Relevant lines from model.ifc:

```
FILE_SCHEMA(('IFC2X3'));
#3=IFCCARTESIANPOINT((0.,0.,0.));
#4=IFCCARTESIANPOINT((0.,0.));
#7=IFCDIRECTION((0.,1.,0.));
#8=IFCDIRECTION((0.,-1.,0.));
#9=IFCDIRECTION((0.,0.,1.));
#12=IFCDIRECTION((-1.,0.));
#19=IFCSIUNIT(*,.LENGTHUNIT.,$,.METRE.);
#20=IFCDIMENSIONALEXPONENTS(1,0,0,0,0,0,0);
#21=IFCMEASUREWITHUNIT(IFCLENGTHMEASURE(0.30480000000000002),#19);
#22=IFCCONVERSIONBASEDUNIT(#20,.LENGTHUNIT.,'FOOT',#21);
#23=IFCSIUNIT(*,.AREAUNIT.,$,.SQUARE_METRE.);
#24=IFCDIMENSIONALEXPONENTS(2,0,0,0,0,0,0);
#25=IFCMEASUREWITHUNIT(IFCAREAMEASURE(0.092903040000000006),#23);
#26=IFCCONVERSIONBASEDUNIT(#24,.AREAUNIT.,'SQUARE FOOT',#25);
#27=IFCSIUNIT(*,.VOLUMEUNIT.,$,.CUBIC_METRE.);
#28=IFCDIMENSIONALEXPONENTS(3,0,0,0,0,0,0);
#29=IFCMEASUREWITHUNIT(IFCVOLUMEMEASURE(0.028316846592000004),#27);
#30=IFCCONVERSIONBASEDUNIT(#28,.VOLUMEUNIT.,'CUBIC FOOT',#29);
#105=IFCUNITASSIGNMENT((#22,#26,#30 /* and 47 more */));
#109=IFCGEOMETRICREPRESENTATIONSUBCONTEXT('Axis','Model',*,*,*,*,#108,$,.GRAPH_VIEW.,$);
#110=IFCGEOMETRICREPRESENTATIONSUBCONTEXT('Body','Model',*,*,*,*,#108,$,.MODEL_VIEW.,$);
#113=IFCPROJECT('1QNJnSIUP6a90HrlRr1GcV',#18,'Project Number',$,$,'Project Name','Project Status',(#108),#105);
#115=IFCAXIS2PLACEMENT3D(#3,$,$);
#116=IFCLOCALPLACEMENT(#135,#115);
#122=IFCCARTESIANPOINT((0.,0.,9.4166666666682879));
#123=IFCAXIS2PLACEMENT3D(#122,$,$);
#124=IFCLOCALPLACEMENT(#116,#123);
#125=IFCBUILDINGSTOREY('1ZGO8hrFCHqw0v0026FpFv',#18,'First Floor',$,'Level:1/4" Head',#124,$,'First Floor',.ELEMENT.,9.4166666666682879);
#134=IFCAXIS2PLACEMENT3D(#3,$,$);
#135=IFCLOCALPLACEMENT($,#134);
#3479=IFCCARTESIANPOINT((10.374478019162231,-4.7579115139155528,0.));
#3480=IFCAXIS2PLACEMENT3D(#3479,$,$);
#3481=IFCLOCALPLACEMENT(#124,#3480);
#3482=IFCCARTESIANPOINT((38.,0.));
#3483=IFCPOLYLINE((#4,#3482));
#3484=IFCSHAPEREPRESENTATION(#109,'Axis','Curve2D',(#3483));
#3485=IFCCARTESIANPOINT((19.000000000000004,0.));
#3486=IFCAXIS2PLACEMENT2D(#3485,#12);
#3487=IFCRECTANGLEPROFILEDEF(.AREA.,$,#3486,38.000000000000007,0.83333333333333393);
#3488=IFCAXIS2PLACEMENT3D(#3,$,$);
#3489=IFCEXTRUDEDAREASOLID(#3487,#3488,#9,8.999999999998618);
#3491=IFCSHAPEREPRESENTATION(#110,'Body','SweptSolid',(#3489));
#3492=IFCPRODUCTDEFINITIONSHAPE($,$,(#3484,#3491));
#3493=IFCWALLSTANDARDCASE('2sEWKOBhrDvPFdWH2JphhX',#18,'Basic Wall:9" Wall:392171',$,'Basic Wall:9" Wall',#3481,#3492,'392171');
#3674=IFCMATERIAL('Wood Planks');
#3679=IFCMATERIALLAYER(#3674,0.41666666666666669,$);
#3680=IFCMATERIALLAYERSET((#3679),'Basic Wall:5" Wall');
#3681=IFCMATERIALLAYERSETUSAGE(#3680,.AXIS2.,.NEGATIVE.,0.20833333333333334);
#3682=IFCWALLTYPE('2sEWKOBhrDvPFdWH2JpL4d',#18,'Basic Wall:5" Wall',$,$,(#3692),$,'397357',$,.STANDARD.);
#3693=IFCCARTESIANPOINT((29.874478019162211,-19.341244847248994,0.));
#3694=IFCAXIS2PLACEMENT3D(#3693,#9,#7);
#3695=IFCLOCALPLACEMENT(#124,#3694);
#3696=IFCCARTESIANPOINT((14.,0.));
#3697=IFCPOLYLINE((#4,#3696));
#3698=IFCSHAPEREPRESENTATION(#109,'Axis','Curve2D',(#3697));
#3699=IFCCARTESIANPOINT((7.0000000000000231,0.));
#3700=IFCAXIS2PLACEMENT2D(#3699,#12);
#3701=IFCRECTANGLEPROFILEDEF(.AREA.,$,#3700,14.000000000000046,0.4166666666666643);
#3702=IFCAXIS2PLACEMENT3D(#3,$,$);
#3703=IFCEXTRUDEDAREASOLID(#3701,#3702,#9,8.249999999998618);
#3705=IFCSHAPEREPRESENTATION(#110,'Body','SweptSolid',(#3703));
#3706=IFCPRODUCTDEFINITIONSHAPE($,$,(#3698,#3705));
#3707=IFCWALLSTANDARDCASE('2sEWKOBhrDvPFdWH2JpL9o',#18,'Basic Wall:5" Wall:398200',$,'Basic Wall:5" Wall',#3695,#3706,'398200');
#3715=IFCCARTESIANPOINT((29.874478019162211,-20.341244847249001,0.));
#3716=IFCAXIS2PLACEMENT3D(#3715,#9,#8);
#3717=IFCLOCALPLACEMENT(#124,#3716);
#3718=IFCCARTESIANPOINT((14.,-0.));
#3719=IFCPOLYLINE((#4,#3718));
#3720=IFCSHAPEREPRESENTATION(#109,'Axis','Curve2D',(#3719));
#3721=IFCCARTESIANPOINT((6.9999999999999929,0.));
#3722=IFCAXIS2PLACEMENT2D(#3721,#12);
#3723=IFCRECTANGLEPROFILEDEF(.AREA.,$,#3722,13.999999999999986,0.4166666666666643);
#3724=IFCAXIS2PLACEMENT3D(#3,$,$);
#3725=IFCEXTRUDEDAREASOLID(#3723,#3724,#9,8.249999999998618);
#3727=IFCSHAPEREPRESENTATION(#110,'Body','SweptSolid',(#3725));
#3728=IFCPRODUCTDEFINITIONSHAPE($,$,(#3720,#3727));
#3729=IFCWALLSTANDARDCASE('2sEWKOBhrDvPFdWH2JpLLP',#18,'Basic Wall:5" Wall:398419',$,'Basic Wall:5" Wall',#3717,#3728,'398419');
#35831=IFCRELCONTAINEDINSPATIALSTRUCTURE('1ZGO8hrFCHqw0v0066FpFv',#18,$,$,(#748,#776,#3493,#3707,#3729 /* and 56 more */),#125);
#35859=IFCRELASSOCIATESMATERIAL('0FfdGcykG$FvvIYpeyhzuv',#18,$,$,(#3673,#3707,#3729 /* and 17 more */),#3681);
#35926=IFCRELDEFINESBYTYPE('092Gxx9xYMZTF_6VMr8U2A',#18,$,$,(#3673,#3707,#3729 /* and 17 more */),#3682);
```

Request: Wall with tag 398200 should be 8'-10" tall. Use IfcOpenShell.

```python
import ifcopenshell
import ifcopenshell.geom
import ifcopenshell.util.representation
import ifcopenshell.util.shape
import ifcopenshell.util.unit

model = ifcopenshell.open("model.ifc")
unit_scale = ifcopenshell.util.unit.calculate_unit_scale(model)
settings = ifcopenshell.geom.settings()


def volume(element):
    """Net volume in cubic metres, openings subtracted."""
    shape = ifcopenshell.geom.create_shape(settings, element)
    return ifcopenshell.util.shape.get_volume(shape.geometry)


wall = model.by_guid("2sEWKOBhrDvPFdWH2JpL9o")
before = volume(wall)

body = ifcopenshell.util.representation.get_representation(wall, "Model", "Body")
solid = body.Items[0]
old_height = solid.Depth
solid.Depth = 106 * 0.0254 / unit_scale
after = volume(wall)

print(f"height {old_height:g} -> {solid.Depth:g}, volume {before:.3f} -> {after:.3f} m3")

model.write("model_updated.ifc")
```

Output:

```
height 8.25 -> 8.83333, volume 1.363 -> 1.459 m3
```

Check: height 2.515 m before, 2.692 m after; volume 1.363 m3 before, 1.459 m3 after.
